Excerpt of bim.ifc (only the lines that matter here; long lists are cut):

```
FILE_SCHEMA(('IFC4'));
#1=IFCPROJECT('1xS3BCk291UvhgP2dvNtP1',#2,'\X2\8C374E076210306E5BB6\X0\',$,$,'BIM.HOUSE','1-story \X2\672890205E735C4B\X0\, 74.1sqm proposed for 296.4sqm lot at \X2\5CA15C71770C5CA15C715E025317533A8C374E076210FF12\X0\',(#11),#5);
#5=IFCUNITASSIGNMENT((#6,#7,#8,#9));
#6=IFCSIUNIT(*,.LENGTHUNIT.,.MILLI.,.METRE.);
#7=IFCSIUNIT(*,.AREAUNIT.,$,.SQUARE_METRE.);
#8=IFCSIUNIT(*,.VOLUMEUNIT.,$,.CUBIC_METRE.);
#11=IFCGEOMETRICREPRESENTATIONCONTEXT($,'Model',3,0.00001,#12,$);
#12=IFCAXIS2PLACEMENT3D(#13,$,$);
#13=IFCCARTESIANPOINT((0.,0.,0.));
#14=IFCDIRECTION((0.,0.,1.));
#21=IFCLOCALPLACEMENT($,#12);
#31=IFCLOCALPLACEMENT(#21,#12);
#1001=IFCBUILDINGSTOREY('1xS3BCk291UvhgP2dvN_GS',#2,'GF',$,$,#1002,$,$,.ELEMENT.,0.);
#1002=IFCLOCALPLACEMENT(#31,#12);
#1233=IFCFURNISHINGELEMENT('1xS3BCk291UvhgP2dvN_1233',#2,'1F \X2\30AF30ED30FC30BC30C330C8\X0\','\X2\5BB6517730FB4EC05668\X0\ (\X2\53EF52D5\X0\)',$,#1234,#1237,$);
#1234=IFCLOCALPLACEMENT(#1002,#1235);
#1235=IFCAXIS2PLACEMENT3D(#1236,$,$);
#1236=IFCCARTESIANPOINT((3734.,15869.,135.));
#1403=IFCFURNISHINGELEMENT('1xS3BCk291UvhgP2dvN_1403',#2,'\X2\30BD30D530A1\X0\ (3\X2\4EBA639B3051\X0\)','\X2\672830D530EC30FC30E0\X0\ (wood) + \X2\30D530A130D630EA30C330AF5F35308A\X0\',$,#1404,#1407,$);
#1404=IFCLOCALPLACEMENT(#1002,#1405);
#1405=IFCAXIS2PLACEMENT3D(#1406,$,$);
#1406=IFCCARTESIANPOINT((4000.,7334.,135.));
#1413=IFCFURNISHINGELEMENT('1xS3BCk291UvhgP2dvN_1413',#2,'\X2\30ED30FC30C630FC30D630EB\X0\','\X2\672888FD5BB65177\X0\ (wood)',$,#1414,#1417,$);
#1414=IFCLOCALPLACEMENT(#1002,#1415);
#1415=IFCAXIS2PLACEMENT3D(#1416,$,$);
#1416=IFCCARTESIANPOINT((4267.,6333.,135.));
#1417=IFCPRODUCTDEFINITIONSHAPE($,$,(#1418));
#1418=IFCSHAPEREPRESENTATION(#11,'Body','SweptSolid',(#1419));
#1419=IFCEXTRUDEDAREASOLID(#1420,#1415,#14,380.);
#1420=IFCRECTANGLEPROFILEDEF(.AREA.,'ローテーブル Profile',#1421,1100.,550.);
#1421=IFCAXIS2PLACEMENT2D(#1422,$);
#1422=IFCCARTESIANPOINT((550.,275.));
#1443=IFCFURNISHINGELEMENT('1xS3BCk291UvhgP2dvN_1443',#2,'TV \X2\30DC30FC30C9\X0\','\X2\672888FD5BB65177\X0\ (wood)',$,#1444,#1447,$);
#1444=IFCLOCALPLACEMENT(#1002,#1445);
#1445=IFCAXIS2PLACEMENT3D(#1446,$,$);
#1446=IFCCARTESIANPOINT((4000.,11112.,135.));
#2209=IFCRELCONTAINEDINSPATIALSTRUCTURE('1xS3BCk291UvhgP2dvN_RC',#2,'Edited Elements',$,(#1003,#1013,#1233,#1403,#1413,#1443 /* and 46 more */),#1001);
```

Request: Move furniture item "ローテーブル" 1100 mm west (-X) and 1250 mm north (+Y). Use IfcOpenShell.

```python
import ifcopenshell
import ifcopenshell.api.geometry
import ifcopenshell.util.placement
import ifcopenshell.util.unit

model = ifcopenshell.open("bim.ifc")
unit_scale = ifcopenshell.util.unit.calculate_unit_scale(model)

item = model.by_id(1413)
matrix = ifcopenshell.util.placement.get_local_placement(item.ObjectPlacement)
matrix[0, 3] -= 1.1 / unit_scale
matrix[1, 3] += 1.25 / unit_scale
ifcopenshell.api.geometry.edit_object_placement(model, product=item, matrix=matrix, is_si=False)

print(ifcopenshell.util.placement.get_local_placement(item.ObjectPlacement).round(3) + 0.0)

model.write("bim_edited.ifc")
```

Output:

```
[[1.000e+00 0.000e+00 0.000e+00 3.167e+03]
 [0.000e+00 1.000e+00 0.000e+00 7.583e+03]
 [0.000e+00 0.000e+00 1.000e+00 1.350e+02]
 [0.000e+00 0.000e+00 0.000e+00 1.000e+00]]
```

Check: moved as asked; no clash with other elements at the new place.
